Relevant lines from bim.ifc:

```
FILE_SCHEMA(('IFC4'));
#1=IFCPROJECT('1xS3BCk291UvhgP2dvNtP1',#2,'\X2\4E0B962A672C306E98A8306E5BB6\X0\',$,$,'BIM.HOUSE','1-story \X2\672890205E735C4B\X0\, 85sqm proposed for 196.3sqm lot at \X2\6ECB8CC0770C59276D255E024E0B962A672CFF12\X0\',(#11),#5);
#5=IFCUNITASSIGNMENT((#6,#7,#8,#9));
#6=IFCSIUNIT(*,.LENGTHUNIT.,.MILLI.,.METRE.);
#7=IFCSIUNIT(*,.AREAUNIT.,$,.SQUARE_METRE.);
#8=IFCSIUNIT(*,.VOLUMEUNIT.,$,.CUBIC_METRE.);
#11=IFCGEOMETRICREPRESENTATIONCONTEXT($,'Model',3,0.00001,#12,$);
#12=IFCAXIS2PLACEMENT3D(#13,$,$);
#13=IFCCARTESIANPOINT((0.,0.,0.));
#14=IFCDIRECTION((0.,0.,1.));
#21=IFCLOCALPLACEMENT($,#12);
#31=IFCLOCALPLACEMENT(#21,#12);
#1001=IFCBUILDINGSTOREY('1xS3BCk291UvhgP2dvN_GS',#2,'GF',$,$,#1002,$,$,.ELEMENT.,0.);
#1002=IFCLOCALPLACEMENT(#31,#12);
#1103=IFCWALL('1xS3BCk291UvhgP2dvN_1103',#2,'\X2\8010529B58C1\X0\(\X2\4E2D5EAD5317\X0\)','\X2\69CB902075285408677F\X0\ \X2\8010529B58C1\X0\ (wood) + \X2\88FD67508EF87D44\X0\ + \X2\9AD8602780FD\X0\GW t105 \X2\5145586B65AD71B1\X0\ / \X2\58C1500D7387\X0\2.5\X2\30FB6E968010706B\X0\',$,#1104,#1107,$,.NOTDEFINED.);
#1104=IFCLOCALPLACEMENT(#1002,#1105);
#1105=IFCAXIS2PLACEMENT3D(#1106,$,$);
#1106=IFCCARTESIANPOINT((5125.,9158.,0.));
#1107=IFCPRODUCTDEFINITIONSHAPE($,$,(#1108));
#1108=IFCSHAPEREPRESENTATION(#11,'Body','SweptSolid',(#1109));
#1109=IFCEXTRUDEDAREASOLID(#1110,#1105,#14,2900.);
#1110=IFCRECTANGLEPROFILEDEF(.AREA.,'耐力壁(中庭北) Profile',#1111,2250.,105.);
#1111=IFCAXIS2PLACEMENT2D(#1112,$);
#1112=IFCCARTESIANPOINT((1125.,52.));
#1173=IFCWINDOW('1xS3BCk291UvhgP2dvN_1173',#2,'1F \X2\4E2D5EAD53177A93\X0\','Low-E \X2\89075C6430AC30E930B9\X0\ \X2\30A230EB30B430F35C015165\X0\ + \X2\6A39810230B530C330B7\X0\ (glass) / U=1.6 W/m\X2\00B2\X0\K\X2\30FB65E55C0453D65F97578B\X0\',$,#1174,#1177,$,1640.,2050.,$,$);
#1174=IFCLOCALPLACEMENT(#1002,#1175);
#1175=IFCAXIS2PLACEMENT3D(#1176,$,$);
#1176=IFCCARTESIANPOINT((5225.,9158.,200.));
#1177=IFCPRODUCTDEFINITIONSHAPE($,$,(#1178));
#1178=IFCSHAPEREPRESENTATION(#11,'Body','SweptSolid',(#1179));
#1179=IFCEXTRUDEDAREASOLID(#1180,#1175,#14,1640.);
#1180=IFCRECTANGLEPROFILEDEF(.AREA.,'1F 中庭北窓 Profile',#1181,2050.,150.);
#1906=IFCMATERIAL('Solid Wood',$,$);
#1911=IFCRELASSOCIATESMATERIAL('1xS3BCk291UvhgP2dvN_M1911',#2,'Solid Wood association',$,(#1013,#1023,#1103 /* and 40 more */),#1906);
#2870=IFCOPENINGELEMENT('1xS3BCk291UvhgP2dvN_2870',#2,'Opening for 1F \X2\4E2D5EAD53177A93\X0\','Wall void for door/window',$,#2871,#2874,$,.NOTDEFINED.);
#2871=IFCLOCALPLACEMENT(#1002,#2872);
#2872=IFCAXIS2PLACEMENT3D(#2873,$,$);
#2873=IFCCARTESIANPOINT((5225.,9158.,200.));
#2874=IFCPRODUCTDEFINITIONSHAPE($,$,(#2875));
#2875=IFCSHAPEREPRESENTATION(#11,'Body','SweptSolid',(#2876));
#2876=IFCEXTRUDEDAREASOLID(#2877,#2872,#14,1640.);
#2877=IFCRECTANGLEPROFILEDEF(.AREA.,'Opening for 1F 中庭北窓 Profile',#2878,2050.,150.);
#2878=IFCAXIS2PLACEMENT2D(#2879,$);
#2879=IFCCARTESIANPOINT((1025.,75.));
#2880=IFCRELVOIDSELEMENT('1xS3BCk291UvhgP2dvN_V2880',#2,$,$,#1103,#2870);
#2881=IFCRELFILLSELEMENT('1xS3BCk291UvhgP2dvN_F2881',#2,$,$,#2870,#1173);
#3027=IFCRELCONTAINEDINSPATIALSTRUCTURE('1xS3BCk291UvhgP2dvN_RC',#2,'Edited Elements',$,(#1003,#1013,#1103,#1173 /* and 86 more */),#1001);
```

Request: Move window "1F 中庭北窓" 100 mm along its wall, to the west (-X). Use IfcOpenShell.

```python
import ifcopenshell
import ifcopenshell.api.geometry
import ifcopenshell.util.placement
import ifcopenshell.util.unit

model = ifcopenshell.open("bim.ifc")
unit_scale = ifcopenshell.util.unit.calculate_unit_scale(model)

window = model.by_id(1173)
opening = window.FillsVoids[0].RelatingOpeningElement
wall = opening.VoidsElements[0].RelatingBuildingElement

wall_matrix = ifcopenshell.util.placement.get_local_placement(wall.ObjectPlacement)
shift = wall_matrix[:3, 0] * -0.1 / unit_scale
before = ifcopenshell.util.placement.get_local_placement(window.ObjectPlacement)[:3, 3].copy()

# The window is not placed relative to its opening, so move both.
for product in (opening, window):
    matrix = ifcopenshell.util.placement.get_local_placement(product.ObjectPlacement)
    matrix[:3, 3] += shift
    ifcopenshell.api.geometry.edit_object_placement(model, product=product, matrix=matrix, is_si=False)

after = ifcopenshell.util.placement.get_local_placement(window.ObjectPlacement)[:3, 3]
print("window moved by", (after - before).round(3) + 0.0)

model.write("bim_v2.ifc")
```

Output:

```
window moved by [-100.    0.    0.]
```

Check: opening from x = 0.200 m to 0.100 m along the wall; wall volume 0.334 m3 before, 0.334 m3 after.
